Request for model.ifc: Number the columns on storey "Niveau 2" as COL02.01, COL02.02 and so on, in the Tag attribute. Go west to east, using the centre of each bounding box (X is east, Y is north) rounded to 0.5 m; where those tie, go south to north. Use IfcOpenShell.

First a look at what the model holds.

```python
import ifcopenshell
import ifcopenshell.util.element
import ifcopenshell.util.placement

model = ifcopenshell.open("model.ifc")
print(model.schema)
storey = next(s for s in model.by_type("IfcBuildingStorey") if s.Name == "Niveau 2")
columns = [e for e in ifcopenshell.util.element.get_decomposition(storey) if e.is_a("IfcColumn")]
for e in sorted(columns, key=lambda e: e.id()):
    origin = ifcopenshell.util.placement.get_local_placement(e.ObjectPlacement)[:3, 3]
    print(e.id(), e.Tag, e.Name, origin.round(2) + 0.0, sep=" | ")
```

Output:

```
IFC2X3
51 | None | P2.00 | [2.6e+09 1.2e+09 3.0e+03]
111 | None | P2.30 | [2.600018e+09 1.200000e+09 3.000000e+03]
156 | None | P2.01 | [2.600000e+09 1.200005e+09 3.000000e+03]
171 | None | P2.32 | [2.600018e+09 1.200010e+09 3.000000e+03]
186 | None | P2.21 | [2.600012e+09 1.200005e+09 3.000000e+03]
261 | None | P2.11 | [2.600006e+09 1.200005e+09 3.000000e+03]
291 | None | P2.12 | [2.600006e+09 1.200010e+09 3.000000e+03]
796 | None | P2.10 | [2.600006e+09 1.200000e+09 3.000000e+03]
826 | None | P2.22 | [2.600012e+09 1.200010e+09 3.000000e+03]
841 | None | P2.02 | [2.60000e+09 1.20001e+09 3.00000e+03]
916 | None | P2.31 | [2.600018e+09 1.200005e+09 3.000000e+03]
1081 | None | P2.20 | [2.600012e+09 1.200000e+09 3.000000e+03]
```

```python
import ifcopenshell
import ifcopenshell.geom
import ifcopenshell.util.element
import ifcopenshell.util.shape

model = ifcopenshell.open("model.ifc")
settings = ifcopenshell.geom.settings()
settings.set("use-world-coords", True)


def centre(element):
    shape = ifcopenshell.geom.create_shape(settings, element)
    return ifcopenshell.util.shape.get_bbox_centroid(shape.geometry)


storey = next(s for s in model.by_type("IfcBuildingStorey") if s.Name == "Niveau 2")
columns = [e for e in ifcopenshell.util.element.get_decomposition(storey) if e.is_a("IfcColumn")]

# Insertion points can sit at a corner or the storey origin, so sort by the geometry (in metres).
centres = {e: centre(e) for e in columns}
columns.sort(key=lambda e: (round(centres[e][0] / 0.5), centres[e][1]))

for i, e in enumerate(columns, start=1):
    number = f"COL02.{i:02d}"
    e.Tag = number
    print(e.id(), number)

model.write("model-out.ifc")
```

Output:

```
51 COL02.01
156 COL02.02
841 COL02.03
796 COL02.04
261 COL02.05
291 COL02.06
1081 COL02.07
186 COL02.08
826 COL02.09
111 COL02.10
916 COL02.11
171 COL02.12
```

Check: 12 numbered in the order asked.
